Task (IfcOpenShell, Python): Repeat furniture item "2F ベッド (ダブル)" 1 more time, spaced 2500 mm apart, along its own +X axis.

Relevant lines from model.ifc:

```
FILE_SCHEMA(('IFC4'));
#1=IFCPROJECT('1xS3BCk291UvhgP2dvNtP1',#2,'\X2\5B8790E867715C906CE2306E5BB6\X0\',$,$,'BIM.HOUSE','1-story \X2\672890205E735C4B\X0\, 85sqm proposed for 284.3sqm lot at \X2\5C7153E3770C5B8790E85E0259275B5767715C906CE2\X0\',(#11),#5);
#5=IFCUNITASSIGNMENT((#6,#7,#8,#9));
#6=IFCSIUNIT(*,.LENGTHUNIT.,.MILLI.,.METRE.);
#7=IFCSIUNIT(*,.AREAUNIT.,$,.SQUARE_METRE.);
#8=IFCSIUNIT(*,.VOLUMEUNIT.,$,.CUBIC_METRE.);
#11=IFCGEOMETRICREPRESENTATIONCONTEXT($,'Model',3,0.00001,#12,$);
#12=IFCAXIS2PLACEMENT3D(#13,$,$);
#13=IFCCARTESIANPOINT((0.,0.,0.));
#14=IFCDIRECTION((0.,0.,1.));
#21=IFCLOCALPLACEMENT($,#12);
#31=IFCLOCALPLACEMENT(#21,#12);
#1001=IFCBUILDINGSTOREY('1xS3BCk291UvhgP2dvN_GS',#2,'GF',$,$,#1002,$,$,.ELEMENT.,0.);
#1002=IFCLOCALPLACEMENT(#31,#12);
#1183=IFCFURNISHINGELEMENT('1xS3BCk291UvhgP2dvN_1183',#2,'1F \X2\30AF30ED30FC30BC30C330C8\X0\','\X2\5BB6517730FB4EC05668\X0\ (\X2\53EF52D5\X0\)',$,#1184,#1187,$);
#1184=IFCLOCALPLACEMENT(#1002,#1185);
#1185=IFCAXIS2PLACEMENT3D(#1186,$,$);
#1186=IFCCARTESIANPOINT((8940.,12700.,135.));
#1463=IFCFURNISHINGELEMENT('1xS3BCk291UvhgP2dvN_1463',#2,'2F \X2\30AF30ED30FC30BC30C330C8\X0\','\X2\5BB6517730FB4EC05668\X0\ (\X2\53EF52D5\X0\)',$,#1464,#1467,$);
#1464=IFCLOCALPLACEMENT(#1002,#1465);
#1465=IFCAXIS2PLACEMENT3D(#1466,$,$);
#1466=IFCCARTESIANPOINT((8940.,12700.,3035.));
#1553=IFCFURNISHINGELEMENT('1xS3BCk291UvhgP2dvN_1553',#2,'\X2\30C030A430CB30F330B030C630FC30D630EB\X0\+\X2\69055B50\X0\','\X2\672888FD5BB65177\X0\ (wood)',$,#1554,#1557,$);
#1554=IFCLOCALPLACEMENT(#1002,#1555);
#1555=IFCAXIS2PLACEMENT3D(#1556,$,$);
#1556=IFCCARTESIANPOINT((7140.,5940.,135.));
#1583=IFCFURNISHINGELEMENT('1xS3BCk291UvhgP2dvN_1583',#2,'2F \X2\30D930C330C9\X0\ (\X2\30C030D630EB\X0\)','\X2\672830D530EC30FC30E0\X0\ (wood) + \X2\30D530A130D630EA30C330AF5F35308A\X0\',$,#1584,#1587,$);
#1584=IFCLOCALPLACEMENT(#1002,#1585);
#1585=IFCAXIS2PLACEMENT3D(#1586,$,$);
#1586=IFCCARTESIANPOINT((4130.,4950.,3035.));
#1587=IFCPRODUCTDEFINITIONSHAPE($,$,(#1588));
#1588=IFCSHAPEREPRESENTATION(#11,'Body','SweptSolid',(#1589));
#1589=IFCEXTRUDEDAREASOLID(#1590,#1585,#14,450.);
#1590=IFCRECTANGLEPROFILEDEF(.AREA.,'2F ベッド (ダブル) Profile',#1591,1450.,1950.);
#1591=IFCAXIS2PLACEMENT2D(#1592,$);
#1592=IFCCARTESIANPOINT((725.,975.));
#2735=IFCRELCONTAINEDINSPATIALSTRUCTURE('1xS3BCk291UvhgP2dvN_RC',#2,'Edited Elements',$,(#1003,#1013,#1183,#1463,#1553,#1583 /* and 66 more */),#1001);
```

```python
import ifcopenshell
import ifcopenshell.api.geometry
import ifcopenshell.api.root
import ifcopenshell.util.element
import ifcopenshell.util.placement

model = ifcopenshell.open("model.ifc")


def reuse_history(source, copy):
    """copy_class also copies each property set's owner history, people and application; keep the originals."""
    for rel in copy.IsDefinedBy:
        if rel.is_a("IfcRelDefinesByProperties") and (history := rel.RelatingPropertyDefinition.OwnerHistory):
            rel.RelatingPropertyDefinition.OwnerHistory = source.OwnerHistory
            ifcopenshell.util.element.remove_deep2(model, history)


source = model.by_guid("1xS3BCk291UvhgP2dvN_1583")
base = ifcopenshell.util.placement.get_local_placement(source.ObjectPlacement)
step = base[:3, 0] * 2500.0

for i in range(1, 2):
    copy = ifcopenshell.api.root.copy_class(model, product=source)
    copy.Representation = ifcopenshell.util.element.copy_deep(
        model, source.Representation, exclude=["IfcGeometricRepresentationContext", "IfcRepresentationMap"]
    )
    reuse_history(source, copy)
    matrix = base.copy()
    matrix[:3, 3] += i * step
    print("added at", matrix[:3, 3].round(3) + 0.0)
    ifcopenshell.api.geometry.edit_object_placement(model, product=copy, matrix=matrix, is_si=False)

model.write("model_edited.ifc")
```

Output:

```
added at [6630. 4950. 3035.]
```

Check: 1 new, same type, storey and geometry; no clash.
